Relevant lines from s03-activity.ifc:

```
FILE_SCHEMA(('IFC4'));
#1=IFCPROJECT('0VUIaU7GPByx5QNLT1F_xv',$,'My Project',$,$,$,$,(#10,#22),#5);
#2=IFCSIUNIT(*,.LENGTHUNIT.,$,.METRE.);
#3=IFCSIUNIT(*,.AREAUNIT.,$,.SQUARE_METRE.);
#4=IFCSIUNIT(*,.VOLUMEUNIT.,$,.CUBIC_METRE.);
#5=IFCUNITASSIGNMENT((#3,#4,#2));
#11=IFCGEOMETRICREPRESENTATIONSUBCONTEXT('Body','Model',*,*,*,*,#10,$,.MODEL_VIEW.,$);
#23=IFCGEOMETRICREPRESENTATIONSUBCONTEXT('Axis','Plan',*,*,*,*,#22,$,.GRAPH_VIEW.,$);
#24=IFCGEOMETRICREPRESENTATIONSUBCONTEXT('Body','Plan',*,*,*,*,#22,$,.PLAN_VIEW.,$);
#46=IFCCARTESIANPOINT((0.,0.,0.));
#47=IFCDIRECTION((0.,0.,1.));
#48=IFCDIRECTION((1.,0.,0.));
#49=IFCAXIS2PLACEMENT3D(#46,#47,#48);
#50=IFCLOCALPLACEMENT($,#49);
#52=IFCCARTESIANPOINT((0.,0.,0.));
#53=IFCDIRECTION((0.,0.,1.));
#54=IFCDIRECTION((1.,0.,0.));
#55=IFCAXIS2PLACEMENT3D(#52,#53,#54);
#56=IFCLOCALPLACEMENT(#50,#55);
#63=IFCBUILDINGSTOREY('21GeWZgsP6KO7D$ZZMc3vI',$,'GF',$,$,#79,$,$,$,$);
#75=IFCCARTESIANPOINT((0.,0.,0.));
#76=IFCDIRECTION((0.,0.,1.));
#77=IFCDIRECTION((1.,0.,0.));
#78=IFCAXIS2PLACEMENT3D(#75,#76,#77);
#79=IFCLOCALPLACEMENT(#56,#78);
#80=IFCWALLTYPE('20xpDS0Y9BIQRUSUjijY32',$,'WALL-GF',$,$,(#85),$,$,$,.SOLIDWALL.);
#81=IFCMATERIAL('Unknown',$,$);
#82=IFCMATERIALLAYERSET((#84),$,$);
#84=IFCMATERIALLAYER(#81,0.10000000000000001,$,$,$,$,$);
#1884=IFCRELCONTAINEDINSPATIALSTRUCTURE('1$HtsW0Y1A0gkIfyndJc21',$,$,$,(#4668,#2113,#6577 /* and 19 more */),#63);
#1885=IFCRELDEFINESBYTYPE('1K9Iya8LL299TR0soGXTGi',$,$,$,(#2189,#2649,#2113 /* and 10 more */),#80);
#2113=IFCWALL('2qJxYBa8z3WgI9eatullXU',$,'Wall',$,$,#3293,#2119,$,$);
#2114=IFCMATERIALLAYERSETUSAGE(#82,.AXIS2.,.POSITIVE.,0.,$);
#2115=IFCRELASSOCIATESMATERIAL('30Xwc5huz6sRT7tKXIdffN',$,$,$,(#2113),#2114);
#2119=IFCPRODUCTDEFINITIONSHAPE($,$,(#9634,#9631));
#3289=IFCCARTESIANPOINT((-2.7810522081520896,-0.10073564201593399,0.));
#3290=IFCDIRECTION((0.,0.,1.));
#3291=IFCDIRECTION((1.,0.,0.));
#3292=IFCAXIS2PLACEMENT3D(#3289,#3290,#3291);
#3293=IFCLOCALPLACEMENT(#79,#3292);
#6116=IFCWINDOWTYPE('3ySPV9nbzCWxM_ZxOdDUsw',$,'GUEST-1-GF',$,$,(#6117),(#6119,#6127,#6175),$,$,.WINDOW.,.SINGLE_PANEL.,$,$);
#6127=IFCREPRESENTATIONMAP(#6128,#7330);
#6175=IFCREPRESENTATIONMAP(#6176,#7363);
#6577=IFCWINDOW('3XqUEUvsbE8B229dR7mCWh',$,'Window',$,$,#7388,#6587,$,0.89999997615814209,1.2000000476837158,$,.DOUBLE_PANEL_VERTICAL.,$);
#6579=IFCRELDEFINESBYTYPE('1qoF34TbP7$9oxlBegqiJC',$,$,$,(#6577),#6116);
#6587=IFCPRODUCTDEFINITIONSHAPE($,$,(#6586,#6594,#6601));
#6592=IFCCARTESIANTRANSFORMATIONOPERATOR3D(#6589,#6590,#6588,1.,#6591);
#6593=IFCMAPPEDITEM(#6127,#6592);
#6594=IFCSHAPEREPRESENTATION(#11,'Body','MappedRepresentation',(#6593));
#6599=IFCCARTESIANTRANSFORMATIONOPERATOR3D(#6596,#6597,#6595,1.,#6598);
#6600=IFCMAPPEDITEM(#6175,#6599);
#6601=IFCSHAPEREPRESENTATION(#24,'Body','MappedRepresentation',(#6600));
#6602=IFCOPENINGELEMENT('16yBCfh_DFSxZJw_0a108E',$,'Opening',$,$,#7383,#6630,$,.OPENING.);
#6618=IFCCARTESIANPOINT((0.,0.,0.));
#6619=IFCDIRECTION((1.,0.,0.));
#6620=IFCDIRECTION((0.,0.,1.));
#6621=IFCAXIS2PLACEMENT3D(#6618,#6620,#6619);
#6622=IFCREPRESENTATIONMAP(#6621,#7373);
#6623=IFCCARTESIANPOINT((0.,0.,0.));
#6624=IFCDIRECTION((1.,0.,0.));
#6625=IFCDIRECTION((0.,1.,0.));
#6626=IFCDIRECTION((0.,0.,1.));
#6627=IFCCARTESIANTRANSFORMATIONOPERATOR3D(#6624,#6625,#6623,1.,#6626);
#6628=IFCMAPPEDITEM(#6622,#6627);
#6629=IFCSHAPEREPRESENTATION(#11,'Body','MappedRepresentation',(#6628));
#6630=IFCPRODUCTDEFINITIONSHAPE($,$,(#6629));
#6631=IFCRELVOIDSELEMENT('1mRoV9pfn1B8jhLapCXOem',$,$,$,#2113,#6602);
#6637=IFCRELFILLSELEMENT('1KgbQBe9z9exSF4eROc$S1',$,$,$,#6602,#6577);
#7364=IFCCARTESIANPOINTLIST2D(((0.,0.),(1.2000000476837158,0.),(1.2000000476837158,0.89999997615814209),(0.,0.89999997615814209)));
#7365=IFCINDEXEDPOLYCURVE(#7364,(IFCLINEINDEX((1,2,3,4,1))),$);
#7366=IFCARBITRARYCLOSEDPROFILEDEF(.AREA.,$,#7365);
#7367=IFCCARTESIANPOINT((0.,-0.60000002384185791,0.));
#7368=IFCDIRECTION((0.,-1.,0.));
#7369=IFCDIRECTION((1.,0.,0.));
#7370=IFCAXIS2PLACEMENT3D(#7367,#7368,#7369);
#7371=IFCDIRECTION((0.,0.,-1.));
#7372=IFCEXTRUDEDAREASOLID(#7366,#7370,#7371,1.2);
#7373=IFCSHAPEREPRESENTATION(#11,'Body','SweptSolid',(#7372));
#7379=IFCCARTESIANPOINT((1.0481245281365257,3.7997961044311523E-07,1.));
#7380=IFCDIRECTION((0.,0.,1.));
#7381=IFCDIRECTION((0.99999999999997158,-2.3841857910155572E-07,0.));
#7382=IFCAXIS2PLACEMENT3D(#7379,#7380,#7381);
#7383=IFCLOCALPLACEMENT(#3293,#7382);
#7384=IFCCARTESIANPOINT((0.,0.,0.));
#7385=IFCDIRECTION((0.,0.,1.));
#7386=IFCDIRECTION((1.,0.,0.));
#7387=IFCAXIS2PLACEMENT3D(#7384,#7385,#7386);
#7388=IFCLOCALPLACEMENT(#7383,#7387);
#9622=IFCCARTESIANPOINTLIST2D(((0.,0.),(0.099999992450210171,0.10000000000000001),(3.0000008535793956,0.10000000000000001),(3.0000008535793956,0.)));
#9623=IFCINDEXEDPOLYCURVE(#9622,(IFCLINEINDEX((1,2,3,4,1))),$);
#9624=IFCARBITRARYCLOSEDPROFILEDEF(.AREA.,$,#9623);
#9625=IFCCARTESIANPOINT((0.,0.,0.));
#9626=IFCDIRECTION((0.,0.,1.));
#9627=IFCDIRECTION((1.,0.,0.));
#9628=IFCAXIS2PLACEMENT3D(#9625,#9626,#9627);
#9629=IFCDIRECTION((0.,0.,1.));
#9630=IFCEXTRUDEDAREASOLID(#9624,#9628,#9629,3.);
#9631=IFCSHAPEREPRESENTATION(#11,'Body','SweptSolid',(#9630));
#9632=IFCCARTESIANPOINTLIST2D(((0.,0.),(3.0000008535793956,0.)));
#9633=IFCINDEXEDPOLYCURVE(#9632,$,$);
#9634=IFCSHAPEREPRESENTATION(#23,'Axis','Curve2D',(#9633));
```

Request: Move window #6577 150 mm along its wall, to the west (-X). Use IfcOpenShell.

```python
import ifcopenshell
import ifcopenshell.api.geometry
import ifcopenshell.util.placement
import ifcopenshell.util.unit

model = ifcopenshell.open("s03-activity.ifc")
unit_scale = ifcopenshell.util.unit.calculate_unit_scale(model)

window = model.by_guid("3XqUEUvsbE8B229dR7mCWh")
opening = window.FillsVoids[0].RelatingOpeningElement
wall = opening.VoidsElements[0].RelatingBuildingElement

wall_matrix = ifcopenshell.util.placement.get_local_placement(wall.ObjectPlacement)
shift = wall_matrix[:3, 0] * -0.15 / unit_scale
before = ifcopenshell.util.placement.get_local_placement(window.ObjectPlacement)[:3, 3].copy()

# The window is placed relative to its opening, so it follows when the opening moves.
matrix = ifcopenshell.util.placement.get_local_placement(opening.ObjectPlacement)
matrix[:3, 3] += shift
ifcopenshell.api.geometry.edit_object_placement(
    model, product=opening, matrix=matrix, is_si=False, should_transform_children=True
)

after = ifcopenshell.util.placement.get_local_placement(window.ObjectPlacement)[:3, 3]
print("window moved by", (after - before).round(3) + 0.0)

model.write("s03-activity_edited.ifc")
```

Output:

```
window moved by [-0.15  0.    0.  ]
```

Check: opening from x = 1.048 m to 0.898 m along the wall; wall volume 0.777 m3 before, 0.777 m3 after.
